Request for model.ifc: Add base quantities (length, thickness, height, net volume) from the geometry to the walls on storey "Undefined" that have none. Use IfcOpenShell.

First a look at what the model holds.

```python
import ifcopenshell
import ifcopenshell.util.element
import ifcopenshell.util.unit

model = ifcopenshell.open("model.ifc")
print(model.schema)
for unit_type in ("LENGTHUNIT", "AREAUNIT", "VOLUMEUNIT"):
    print(unit_type, ifcopenshell.util.unit.calculate_unit_scale(model, unit_type))
storey = next(s for s in model.by_type("IfcBuildingStorey") if s.Name == "Undefined")
walls = [e for e in ifcopenshell.util.element.get_decomposition(storey) if e.is_a("IfcWall")]
for e in sorted(walls, key=lambda e: e.id()):
    print(e.id(), e.is_a(), e.Name, list(ifcopenshell.util.element.get_psets(e, qtos_only=True)), sep=" | ")
```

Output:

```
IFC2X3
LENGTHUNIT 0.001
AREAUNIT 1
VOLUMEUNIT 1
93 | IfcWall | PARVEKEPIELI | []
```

```python
import ifcopenshell
import ifcopenshell.api.pset
import ifcopenshell.geom
import ifcopenshell.util.element
import ifcopenshell.util.shape
import ifcopenshell.util.unit

model = ifcopenshell.open("model.ifc")
unit_scale = ifcopenshell.util.unit.calculate_unit_scale(model)
volume_scale = ifcopenshell.util.unit.calculate_unit_scale(model, "VOLUMEUNIT")
settings = ifcopenshell.geom.settings()

storey = next(s for s in model.by_type("IfcBuildingStorey") if s.Name == "Undefined")
walls = [e for e in ifcopenshell.util.element.get_decomposition(storey) if e.is_a("IfcWall")]

for e in sorted(walls, key=lambda e: e.id()):
    if ifcopenshell.util.element.get_psets(e, qtos_only=True, should_inherit=False):
        continue
    # Geometry comes back in metres, in the element's own axes.
    shape = ifcopenshell.geom.create_shape(settings, e)
    values = {
        "Length": ifcopenshell.util.shape.get_x(shape.geometry) / unit_scale,
        "Width": ifcopenshell.util.shape.get_y(shape.geometry) / unit_scale,
        "Height": ifcopenshell.util.shape.get_z(shape.geometry) / unit_scale,
        "NetVolume": ifcopenshell.util.shape.get_volume(shape.geometry) / volume_scale,
    }
    qto = ifcopenshell.api.pset.add_qto(model, product=e, name="BaseQuantities")
    ifcopenshell.api.pset.edit_qto(model, qto=qto, properties=values)
    print(e.id(), {k: round(v, 3) for k, v in values.items()})

model.write("model_edited.ifc")
```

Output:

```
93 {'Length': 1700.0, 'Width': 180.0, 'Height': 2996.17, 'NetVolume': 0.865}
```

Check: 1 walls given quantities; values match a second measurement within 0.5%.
